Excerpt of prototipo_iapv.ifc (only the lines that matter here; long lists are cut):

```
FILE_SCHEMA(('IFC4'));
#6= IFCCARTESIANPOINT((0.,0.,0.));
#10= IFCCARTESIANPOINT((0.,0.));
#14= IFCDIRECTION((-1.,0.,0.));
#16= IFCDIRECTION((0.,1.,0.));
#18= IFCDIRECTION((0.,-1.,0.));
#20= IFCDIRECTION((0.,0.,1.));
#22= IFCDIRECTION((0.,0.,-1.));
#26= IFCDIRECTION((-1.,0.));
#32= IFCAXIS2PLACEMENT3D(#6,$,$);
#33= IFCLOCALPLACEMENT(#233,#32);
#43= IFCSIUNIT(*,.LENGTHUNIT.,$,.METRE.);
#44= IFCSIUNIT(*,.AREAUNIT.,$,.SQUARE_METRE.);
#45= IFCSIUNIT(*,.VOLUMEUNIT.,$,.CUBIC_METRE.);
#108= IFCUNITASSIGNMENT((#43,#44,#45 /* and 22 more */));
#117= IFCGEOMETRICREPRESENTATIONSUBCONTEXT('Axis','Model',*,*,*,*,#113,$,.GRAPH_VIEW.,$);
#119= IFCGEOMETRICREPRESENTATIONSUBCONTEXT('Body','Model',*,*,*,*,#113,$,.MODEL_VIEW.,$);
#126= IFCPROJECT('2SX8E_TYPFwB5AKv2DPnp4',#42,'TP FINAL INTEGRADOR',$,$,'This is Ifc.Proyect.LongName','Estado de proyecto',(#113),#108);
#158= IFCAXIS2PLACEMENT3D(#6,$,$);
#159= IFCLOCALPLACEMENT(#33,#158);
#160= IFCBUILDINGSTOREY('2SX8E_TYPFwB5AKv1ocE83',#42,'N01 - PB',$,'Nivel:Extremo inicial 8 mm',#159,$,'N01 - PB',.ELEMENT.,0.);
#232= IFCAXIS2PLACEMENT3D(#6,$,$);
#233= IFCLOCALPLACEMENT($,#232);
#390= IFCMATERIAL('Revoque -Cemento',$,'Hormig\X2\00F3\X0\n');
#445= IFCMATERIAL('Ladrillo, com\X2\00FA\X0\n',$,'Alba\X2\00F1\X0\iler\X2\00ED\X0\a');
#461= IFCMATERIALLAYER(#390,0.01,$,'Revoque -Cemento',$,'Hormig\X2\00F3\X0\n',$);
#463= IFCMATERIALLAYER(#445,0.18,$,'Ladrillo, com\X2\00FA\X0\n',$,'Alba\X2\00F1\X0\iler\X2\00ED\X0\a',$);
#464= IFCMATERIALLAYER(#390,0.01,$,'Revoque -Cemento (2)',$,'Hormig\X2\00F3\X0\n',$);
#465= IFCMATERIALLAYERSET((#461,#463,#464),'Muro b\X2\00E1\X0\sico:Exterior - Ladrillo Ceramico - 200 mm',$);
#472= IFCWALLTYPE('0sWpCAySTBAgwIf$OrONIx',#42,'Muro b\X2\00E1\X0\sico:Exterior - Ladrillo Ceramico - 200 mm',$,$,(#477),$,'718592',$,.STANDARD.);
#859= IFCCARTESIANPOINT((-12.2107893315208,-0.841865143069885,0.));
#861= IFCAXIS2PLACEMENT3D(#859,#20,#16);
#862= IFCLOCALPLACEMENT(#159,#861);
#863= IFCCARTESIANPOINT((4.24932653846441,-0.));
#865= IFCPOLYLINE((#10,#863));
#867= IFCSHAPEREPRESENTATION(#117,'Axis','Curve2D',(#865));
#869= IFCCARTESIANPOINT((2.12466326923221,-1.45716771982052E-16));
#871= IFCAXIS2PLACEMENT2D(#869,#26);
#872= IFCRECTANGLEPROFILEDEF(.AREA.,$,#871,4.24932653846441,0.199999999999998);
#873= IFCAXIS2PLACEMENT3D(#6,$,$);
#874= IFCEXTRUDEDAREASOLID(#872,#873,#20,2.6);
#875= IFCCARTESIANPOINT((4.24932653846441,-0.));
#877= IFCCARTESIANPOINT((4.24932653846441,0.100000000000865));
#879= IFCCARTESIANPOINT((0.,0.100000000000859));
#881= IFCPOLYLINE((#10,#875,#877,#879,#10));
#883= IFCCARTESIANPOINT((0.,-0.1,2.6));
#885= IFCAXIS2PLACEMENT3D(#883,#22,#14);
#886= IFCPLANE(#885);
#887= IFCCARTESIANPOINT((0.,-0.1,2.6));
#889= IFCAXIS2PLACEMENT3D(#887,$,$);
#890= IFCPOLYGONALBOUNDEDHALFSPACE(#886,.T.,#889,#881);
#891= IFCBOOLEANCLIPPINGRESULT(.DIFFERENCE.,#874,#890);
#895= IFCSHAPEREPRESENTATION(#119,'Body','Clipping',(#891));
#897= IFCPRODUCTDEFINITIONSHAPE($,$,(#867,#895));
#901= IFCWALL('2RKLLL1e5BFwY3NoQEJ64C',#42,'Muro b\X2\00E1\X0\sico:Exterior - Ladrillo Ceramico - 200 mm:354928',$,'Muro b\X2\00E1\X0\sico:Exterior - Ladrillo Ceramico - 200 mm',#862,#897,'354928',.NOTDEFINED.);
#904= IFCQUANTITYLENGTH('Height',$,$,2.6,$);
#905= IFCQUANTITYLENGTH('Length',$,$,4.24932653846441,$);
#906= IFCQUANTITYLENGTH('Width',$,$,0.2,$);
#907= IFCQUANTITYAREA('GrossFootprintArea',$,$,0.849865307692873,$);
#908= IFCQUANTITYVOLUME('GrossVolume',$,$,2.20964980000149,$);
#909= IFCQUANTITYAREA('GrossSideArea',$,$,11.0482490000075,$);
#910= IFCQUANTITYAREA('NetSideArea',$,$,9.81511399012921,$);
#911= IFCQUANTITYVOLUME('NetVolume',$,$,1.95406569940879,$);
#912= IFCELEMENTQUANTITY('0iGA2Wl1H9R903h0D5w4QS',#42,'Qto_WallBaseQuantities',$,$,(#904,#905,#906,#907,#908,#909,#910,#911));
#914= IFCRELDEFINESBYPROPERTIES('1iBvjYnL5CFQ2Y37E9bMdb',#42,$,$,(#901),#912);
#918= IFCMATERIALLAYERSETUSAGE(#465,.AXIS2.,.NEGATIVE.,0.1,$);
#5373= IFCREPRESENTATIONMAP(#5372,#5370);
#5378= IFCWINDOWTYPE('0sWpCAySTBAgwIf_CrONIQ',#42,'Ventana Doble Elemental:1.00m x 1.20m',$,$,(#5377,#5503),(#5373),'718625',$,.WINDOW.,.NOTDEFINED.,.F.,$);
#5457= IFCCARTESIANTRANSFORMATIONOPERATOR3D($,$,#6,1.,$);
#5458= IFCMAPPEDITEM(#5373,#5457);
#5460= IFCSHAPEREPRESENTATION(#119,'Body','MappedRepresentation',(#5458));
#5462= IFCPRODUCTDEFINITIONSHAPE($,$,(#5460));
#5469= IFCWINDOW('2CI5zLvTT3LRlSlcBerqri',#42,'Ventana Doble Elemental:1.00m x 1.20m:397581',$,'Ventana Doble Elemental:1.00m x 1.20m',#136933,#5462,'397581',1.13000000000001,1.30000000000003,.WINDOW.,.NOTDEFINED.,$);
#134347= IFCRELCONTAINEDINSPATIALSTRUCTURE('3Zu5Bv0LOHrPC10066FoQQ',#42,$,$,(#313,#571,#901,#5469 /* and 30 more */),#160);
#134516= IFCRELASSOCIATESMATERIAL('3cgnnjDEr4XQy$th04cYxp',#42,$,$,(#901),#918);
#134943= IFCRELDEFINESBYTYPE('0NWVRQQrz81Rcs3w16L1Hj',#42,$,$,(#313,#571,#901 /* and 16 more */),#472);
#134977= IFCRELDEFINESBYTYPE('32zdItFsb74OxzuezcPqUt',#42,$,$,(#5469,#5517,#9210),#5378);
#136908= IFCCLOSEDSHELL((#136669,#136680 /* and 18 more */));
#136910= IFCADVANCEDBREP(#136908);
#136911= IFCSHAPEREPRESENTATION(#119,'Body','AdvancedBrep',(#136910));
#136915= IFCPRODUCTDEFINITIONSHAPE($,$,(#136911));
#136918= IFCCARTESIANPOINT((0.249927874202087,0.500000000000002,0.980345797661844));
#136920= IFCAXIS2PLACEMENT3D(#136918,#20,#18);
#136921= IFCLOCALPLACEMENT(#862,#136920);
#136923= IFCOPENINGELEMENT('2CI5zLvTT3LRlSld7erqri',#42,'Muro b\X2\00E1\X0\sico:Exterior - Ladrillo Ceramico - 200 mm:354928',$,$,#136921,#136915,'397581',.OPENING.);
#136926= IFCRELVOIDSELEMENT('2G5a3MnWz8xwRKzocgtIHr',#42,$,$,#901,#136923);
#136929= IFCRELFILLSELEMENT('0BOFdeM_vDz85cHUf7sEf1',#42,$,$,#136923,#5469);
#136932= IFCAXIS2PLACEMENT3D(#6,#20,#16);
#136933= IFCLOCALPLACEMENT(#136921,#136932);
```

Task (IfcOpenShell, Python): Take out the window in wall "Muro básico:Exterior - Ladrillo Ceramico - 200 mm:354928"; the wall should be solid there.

```python
import ifcopenshell
import ifcopenshell.api.feature
import ifcopenshell.api.pset
import ifcopenshell.api.root
import ifcopenshell.geom
import ifcopenshell.util.element
import ifcopenshell.util.shape
import ifcopenshell.util.unit

model = ifcopenshell.open("prototipo_iapv.ifc")
area_scale = ifcopenshell.util.unit.calculate_unit_scale(model, "AREAUNIT")
volume_scale = ifcopenshell.util.unit.calculate_unit_scale(model, "VOLUMEUNIT")
settings = ifcopenshell.geom.settings()


def volume(element):
    """Net volume in cubic metres, openings subtracted."""
    shape = ifcopenshell.geom.create_shape(settings, element)
    return ifcopenshell.util.shape.get_volume(shape.geometry)


window = model.by_guid("2CI5zLvTT3LRlSlcBerqri")
opening = window.FillsVoids[0].RelatingOpeningElement
wall = opening.VoidsElements[0].RelatingBuildingElement
before = volume(wall)

ifcopenshell.api.root.remove_product(model, product=window)
ifcopenshell.api.feature.remove_feature(model, feature=opening)

after = volume(wall)
thickness = 0.2  # wall thickness in metres

# Update the wall's stored quantities.
qto = model.by_id(ifcopenshell.util.element.get_pset(wall, "Qto_WallBaseQuantities", should_inherit=False)["id"])
ifcopenshell.api.pset.edit_qto(model, qto=qto, properties={
    "NetSideArea": after / thickness / area_scale,
    "NetVolume": after / volume_scale,
})

print(f"wall volume {before:.3f} -> {after:.3f} m3")

model.write("prototipo_iapv_rev.ifc")
```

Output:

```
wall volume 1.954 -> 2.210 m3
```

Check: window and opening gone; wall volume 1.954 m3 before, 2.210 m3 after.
